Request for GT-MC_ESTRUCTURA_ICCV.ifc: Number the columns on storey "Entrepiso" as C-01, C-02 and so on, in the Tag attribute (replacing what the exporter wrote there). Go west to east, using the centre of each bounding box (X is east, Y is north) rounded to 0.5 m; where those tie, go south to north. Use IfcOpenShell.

First a look at what the model holds.

```python
import ifcopenshell
import ifcopenshell.util.element
import ifcopenshell.util.placement

model = ifcopenshell.open("GT-MC_ESTRUCTURA_ICCV.ifc")
print(model.schema)
storey = next(s for s in model.by_type("IfcBuildingStorey") if s.Name == "Entrepiso")
columns = [e for e in ifcopenshell.util.element.get_decomposition(storey) if e.is_a("IfcColumn")]
for e in sorted(columns, key=lambda e: e.id()):
    origin = ifcopenshell.util.placement.get_local_placement(e.ObjectPlacement)[:3, 3]
    print(e.id(), e.Tag, e.Name, origin.round(2) + 0.0, sep=" | ")
```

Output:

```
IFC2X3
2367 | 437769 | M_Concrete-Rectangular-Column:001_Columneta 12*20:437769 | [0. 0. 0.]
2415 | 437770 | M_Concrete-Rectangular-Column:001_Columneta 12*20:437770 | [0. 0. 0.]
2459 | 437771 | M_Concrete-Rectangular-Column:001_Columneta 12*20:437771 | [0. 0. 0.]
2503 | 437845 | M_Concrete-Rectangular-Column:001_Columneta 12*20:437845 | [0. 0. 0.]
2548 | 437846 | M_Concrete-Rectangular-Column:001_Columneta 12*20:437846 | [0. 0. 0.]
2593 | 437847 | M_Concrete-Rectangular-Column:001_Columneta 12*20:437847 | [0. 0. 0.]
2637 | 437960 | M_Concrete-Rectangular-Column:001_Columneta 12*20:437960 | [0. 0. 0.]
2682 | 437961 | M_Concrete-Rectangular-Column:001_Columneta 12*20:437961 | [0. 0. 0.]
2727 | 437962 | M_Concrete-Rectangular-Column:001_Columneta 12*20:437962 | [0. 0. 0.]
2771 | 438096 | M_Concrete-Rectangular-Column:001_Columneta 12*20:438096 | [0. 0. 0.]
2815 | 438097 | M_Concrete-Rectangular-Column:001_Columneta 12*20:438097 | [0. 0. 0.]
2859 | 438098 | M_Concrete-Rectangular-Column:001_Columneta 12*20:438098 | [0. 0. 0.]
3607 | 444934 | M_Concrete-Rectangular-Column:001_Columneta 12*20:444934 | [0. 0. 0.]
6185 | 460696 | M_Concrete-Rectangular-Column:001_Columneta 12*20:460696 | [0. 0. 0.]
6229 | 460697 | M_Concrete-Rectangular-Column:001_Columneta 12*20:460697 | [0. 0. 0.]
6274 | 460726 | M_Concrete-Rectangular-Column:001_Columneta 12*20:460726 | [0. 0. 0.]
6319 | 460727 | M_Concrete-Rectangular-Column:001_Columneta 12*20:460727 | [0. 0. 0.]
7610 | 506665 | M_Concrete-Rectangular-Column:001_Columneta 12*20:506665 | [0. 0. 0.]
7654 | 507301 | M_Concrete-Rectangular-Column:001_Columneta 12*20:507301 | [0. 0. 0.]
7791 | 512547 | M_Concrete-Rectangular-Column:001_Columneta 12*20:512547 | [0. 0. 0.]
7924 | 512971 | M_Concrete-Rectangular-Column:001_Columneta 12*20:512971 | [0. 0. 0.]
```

```python
import ifcopenshell
import ifcopenshell.geom
import ifcopenshell.util.element
import ifcopenshell.util.shape

model = ifcopenshell.open("GT-MC_ESTRUCTURA_ICCV.ifc")
settings = ifcopenshell.geom.settings()
settings.set("use-world-coords", True)


def centre(element):
    shape = ifcopenshell.geom.create_shape(settings, element)
    return ifcopenshell.util.shape.get_bbox_centroid(shape.geometry)


storey = next(s for s in model.by_type("IfcBuildingStorey") if s.Name == "Entrepiso")
columns = [e for e in ifcopenshell.util.element.get_decomposition(storey) if e.is_a("IfcColumn")]

# Insertion points can sit at a corner or the storey origin, so sort by the geometry (in metres).
centres = {e: centre(e) for e in columns}
columns.sort(key=lambda e: (round(centres[e][0] / 0.5), centres[e][1]))

for i, e in enumerate(columns, start=1):
    number = f"C-{i:02d}"
    e.Tag = number
    print(e.id(), number)

model.write("GT-MC_ESTRUCTURA_ICCV_rev.ifc")
```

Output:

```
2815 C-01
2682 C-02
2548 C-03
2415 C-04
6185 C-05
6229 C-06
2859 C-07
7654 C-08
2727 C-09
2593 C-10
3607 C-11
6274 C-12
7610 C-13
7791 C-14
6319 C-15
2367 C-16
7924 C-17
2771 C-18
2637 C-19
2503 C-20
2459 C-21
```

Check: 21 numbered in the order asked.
